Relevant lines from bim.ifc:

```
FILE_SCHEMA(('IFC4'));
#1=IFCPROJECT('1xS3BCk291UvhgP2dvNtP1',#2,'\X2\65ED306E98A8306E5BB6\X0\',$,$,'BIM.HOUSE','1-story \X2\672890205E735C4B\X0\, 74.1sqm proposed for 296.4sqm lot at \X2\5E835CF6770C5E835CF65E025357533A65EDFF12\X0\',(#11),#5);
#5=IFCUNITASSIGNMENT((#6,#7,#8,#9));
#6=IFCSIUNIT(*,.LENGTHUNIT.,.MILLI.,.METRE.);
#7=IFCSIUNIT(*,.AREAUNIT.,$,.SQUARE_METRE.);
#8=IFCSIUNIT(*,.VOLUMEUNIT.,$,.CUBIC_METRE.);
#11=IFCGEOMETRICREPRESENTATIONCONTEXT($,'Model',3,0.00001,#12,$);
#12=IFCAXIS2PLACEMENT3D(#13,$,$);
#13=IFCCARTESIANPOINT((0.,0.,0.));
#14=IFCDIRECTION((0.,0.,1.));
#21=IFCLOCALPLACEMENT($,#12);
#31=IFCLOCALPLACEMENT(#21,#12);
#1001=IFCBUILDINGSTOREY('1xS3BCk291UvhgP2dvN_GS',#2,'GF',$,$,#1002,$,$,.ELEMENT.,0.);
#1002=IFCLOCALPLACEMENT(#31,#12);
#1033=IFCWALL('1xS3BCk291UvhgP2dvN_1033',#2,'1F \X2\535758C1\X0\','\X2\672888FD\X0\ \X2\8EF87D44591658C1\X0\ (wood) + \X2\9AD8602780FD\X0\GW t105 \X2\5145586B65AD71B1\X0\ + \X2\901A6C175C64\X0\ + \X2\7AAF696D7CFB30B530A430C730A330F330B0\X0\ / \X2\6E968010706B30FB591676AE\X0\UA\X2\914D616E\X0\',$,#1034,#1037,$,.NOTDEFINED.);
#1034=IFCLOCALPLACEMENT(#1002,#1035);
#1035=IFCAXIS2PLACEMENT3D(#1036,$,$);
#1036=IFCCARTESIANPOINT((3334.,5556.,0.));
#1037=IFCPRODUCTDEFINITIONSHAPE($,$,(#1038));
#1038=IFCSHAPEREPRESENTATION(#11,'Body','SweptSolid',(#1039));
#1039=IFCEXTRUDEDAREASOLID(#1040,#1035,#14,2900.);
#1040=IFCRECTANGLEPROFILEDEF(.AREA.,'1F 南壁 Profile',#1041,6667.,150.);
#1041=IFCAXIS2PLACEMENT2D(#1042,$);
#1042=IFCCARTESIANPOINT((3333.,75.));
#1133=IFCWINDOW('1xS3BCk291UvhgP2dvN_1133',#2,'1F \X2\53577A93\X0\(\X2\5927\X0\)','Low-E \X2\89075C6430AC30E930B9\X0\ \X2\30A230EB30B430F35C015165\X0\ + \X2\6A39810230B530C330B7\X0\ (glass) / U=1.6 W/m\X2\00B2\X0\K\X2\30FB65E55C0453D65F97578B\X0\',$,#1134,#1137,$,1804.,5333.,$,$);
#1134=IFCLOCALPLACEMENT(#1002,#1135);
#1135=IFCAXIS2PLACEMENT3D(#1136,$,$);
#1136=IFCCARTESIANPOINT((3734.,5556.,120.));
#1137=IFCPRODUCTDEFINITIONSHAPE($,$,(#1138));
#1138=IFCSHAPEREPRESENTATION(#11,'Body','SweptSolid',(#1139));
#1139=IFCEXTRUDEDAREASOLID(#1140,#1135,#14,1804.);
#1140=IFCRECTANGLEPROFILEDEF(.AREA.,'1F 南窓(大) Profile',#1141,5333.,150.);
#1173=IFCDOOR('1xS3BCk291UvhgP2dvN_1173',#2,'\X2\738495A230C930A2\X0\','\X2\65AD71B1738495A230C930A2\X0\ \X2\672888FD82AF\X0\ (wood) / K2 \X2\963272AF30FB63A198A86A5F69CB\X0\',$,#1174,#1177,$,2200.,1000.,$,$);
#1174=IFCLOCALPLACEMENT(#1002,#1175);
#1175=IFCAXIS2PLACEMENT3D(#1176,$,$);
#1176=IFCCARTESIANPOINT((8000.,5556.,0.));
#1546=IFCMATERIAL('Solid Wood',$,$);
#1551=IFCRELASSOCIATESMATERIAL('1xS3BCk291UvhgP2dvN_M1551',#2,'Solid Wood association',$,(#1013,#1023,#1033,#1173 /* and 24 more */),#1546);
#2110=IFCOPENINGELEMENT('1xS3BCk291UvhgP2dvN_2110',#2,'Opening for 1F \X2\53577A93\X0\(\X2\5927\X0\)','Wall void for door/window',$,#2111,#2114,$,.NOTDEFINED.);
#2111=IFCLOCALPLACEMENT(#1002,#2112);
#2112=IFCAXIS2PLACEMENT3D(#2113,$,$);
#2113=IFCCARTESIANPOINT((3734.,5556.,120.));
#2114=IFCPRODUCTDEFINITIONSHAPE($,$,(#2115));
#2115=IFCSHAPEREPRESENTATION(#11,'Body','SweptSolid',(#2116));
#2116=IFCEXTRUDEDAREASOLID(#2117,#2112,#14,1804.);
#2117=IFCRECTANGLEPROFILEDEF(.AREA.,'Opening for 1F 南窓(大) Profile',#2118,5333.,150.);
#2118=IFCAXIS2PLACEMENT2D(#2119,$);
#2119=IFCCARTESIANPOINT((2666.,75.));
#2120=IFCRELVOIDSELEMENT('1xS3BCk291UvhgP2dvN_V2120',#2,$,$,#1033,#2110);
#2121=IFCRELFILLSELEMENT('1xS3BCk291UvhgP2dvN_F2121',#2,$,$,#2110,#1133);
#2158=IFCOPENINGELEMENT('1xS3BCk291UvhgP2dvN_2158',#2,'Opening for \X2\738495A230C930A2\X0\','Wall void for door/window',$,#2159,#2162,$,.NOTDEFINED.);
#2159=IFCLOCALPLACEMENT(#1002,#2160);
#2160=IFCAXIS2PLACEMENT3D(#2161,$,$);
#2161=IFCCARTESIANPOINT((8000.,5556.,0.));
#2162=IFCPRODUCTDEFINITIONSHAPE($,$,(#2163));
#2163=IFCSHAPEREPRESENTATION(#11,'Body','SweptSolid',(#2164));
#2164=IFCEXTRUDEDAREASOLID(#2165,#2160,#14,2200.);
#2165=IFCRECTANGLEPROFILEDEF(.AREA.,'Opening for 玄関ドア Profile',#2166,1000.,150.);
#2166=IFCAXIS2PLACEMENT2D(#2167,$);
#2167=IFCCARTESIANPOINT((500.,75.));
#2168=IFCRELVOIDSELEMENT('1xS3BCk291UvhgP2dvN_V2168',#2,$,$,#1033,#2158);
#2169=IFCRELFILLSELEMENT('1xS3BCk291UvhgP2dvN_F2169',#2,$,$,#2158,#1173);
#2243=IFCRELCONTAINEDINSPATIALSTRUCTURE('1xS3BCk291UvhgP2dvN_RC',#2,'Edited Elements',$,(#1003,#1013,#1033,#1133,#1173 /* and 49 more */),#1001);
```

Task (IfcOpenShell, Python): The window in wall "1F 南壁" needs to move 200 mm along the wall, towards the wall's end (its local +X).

```python
import ifcopenshell
import ifcopenshell.api.geometry
import ifcopenshell.util.placement
import ifcopenshell.util.unit

model = ifcopenshell.open("bim.ifc")
unit_scale = ifcopenshell.util.unit.calculate_unit_scale(model)

window = model.by_guid("1xS3BCk291UvhgP2dvN_1133")
opening = window.FillsVoids[0].RelatingOpeningElement
wall = opening.VoidsElements[0].RelatingBuildingElement

wall_matrix = ifcopenshell.util.placement.get_local_placement(wall.ObjectPlacement)
shift = wall_matrix[:3, 0] * 0.2 / unit_scale
before = ifcopenshell.util.placement.get_local_placement(window.ObjectPlacement)[:3, 3].copy()

# The window is not placed relative to its opening, so move both.
for product in (opening, window):
    matrix = ifcopenshell.util.placement.get_local_placement(product.ObjectPlacement)
    matrix[:3, 3] += shift
    ifcopenshell.api.geometry.edit_object_placement(model, product=product, matrix=matrix, is_si=False)

after = ifcopenshell.util.placement.get_local_placement(window.ObjectPlacement)[:3, 3]
print("window moved by", (after - before).round(3) + 0.0)

model.write("bim_rev.ifc")
```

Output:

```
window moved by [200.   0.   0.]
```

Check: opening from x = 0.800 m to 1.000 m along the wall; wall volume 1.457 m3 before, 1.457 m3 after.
